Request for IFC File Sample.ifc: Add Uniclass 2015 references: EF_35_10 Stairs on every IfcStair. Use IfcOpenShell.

First a look at what the model holds.

```python
import ifcopenshell

model = ifcopenshell.open("IFC File Sample.ifc")
print(model.schema)
print("classifications:", [c.Name for c in model.by_type("IfcClassification")])
for ifc_class in ("IfcDoor", "IfcRoof", "IfcStair", "IfcWall", "IfcWindow"):
    print(ifc_class, len(model.by_type(ifc_class)))
```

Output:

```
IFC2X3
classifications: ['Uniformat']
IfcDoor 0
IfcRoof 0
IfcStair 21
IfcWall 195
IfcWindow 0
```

```python
import ifcopenshell
import ifcopenshell.api.classification

model = ifcopenshell.open("IFC File Sample.ifc")

# IFC2X3 requires Source and Edition and has no link from the project to the system.
system = model.create_entity("IfcClassification", Source="NBS", Edition="2015", Name="Uniclass 2015")

codes = {
    "IfcStair": ("EF_35_10", "Stairs"),
}
for ifc_class, (code, name) in codes.items():
    products = model.by_type(ifc_class)
    ifcopenshell.api.classification.add_reference(
        model, products=products, classification=system, identification=code, name=name
    )
    print(code, len(products))

model.write("IFC File Sample_edited.ifc")
```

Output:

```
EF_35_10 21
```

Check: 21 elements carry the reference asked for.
